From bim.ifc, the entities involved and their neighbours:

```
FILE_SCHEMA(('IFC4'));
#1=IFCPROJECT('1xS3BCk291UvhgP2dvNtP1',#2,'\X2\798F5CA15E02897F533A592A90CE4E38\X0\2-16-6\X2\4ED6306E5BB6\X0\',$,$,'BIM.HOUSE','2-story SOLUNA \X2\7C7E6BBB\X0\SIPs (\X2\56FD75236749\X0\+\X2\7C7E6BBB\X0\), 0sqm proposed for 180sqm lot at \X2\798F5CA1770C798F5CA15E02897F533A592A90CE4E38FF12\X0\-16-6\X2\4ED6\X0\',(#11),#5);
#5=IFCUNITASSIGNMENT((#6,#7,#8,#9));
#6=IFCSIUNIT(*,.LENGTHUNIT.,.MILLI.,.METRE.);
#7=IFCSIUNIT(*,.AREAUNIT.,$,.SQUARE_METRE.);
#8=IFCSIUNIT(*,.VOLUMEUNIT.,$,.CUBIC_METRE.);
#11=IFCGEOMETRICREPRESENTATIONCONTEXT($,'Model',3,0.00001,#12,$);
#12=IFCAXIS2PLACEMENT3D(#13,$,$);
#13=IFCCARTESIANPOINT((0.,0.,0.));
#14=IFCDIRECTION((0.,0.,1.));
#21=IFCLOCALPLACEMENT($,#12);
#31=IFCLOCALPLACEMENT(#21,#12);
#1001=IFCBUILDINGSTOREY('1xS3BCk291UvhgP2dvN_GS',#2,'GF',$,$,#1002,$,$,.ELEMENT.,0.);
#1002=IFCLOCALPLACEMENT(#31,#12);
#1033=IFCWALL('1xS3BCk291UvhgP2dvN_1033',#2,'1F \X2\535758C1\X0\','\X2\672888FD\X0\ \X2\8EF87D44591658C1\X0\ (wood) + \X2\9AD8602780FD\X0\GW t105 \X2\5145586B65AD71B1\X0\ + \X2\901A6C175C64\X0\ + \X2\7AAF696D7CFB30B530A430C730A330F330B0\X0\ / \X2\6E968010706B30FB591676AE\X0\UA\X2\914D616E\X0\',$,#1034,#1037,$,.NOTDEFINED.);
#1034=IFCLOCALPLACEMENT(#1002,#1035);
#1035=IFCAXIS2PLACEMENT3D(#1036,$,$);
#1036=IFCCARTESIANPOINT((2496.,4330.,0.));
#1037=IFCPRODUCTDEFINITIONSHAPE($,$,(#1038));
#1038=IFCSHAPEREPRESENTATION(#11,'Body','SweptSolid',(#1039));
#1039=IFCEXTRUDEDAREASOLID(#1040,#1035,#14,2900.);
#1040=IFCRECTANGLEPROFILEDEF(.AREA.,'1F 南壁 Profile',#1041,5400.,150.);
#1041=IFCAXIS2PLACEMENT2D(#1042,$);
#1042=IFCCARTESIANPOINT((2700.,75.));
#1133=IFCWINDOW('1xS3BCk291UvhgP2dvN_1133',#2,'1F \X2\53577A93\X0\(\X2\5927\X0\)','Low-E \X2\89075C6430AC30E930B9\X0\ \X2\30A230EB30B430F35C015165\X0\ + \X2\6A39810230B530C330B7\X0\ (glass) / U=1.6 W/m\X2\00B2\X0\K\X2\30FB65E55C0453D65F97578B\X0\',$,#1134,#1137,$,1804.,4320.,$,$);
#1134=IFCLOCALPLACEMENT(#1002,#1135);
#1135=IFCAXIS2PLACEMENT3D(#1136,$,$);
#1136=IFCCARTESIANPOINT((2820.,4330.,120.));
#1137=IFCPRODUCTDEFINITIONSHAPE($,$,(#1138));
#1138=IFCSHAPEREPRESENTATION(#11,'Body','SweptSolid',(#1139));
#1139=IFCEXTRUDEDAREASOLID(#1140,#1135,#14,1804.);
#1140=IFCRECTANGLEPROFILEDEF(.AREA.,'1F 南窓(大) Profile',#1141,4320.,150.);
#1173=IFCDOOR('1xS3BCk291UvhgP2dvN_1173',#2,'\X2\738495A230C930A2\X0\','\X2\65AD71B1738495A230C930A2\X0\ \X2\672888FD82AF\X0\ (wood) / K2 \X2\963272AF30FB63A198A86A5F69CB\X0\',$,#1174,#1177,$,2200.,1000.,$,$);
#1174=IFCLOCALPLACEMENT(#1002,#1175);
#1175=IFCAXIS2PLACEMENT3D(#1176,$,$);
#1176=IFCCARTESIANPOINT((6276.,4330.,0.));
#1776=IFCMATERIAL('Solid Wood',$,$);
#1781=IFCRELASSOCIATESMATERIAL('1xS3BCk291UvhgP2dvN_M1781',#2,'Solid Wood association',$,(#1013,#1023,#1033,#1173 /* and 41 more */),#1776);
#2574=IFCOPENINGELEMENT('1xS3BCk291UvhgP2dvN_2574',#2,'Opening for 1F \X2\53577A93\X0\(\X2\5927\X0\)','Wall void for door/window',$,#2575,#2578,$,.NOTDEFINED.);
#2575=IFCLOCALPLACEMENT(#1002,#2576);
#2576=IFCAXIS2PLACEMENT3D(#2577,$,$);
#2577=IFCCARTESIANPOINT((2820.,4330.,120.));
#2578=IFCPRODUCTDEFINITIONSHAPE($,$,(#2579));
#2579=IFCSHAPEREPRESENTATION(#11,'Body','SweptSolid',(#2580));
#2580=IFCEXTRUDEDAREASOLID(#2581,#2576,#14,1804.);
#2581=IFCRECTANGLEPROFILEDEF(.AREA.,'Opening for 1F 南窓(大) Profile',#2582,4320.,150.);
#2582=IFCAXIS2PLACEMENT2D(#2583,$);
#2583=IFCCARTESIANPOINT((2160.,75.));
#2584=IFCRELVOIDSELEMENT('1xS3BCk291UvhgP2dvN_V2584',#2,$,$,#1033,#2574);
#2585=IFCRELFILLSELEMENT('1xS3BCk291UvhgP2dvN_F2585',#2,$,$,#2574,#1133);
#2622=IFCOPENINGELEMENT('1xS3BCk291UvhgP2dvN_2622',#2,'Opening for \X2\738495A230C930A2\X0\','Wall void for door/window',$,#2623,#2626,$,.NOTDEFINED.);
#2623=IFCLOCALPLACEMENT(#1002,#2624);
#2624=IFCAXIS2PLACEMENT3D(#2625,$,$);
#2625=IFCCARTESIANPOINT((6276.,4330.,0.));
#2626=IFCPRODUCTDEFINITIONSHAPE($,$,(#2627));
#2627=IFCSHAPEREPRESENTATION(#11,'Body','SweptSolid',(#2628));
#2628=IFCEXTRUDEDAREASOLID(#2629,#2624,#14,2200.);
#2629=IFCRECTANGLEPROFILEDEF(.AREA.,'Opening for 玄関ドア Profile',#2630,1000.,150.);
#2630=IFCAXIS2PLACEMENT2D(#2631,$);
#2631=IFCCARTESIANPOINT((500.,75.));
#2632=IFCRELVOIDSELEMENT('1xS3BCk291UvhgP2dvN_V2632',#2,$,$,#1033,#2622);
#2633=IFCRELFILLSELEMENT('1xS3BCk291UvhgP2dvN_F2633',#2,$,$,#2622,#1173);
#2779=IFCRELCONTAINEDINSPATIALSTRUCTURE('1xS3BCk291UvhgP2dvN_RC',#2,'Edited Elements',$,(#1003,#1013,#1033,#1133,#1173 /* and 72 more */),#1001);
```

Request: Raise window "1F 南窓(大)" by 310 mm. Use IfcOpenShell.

```python
import numpy as np
import ifcopenshell
import ifcopenshell.api.geometry
import ifcopenshell.util.placement
import ifcopenshell.util.unit

model = ifcopenshell.open("bim.ifc")
unit_scale = ifcopenshell.util.unit.calculate_unit_scale(model)

window = model.by_guid("1xS3BCk291UvhgP2dvN_1133")
opening = window.FillsVoids[0].RelatingOpeningElement
dz = 310.0

shift = np.array([0.0, 0.0, dz])
# The window is not placed relative to its opening, so move both.
for product in (opening, window):
    matrix = ifcopenshell.util.placement.get_local_placement(product.ObjectPlacement)
    matrix[:3, 3] += shift
    ifcopenshell.api.geometry.edit_object_placement(model, product=product, matrix=matrix, is_si=False)

print(f"moved by {dz * unit_scale:+.3f} m")

model.write("bim_edited.ifc")
```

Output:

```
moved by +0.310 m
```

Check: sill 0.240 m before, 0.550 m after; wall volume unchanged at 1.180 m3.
